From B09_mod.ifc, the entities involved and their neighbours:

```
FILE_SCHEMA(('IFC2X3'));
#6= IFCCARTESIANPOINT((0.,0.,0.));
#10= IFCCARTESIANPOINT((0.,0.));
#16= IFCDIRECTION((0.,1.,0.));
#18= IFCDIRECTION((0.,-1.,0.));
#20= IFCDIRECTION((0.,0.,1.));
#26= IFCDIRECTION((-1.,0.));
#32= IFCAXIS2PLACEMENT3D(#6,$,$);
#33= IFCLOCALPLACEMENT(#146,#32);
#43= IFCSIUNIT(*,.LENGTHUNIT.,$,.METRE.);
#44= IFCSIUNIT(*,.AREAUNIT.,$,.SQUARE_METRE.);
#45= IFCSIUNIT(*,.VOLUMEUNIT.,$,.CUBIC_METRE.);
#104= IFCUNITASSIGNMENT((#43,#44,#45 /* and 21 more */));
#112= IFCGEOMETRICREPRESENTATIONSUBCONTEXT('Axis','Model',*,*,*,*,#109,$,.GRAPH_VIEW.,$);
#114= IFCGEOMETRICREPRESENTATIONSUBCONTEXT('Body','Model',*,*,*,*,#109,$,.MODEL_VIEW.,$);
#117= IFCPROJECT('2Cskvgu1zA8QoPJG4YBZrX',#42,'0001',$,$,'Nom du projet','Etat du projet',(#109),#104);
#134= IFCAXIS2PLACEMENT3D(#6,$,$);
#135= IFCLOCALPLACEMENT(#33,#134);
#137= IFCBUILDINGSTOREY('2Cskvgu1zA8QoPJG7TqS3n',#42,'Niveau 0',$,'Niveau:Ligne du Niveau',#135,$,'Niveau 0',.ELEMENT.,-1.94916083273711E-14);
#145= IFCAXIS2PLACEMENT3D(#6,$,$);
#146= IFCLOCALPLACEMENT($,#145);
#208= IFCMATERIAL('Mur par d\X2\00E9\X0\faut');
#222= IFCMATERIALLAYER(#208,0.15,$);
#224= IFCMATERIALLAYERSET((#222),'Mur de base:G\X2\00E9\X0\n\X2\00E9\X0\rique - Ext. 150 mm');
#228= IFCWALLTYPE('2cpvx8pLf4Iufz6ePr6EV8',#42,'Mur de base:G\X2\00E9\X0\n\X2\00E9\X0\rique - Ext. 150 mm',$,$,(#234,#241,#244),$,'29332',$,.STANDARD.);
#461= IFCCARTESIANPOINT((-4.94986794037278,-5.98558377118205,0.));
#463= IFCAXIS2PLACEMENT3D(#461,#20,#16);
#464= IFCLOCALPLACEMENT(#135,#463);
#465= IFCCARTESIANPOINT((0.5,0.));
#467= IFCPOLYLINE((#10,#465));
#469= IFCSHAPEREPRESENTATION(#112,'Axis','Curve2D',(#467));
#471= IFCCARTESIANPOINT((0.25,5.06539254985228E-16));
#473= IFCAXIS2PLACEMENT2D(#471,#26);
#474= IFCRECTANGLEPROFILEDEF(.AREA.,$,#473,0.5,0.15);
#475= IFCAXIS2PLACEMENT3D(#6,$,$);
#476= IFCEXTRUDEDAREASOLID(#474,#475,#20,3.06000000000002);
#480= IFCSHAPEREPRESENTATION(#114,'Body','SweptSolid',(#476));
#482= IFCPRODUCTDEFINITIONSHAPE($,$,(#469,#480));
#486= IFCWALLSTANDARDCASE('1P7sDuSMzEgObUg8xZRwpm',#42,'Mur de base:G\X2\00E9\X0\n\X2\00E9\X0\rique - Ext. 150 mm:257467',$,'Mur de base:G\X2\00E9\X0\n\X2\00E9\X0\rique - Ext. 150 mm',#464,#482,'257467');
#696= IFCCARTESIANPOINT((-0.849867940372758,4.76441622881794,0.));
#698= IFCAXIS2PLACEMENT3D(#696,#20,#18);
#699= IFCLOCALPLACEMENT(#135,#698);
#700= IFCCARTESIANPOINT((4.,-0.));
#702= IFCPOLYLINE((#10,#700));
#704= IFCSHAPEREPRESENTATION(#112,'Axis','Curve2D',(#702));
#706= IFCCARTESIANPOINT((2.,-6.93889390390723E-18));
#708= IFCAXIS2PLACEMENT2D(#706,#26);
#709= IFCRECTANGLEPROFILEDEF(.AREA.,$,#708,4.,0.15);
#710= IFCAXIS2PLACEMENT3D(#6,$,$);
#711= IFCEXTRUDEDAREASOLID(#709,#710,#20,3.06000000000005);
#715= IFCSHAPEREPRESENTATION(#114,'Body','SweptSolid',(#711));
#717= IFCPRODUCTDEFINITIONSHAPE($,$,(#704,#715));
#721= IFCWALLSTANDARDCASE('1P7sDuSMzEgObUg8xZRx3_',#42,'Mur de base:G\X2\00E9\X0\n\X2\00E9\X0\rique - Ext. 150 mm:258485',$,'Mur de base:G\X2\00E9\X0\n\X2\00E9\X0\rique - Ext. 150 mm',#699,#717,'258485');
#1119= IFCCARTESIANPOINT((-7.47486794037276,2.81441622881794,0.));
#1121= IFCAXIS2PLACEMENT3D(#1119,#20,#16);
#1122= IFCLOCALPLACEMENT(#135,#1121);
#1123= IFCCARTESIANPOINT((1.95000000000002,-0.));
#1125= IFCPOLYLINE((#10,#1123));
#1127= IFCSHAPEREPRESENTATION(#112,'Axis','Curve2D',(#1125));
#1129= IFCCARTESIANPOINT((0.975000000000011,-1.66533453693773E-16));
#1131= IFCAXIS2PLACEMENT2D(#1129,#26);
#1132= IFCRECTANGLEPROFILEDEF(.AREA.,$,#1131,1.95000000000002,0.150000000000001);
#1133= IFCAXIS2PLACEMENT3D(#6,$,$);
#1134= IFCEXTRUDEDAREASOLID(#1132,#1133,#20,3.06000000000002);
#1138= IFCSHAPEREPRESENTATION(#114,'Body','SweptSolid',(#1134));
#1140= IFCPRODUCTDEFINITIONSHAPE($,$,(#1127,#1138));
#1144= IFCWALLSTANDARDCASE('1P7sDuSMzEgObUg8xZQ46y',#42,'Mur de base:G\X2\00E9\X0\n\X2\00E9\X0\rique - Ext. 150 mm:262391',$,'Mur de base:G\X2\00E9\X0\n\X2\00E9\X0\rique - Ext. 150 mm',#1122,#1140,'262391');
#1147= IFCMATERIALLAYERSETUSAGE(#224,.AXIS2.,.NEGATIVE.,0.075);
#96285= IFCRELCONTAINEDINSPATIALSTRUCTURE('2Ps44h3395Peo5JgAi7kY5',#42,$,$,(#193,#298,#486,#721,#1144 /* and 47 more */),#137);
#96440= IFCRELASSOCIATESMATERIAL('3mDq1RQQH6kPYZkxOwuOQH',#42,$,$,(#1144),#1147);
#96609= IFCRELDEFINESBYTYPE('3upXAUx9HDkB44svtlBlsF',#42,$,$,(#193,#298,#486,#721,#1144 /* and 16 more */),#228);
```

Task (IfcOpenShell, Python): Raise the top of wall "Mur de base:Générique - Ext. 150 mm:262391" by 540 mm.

```python
import ifcopenshell
import ifcopenshell.geom
import ifcopenshell.util.representation
import ifcopenshell.util.shape
import ifcopenshell.util.unit

model = ifcopenshell.open("B09_mod.ifc")
unit_scale = ifcopenshell.util.unit.calculate_unit_scale(model)
settings = ifcopenshell.geom.settings()


def volume(element):
    """Net volume in cubic metres, openings subtracted."""
    shape = ifcopenshell.geom.create_shape(settings, element)
    return ifcopenshell.util.shape.get_volume(shape.geometry)


wall = model.by_guid("1P7sDuSMzEgObUg8xZQ46y")
before = volume(wall)

body = ifcopenshell.util.representation.get_representation(wall, "Model", "Body")
solid = body.Items[0]
old_height = solid.Depth
solid.Depth += 0.54 / unit_scale
after = volume(wall)

print(f"height {old_height:g} -> {solid.Depth:g}, volume {before:.3f} -> {after:.3f} m3")

model.write("B09_mod_edited.ifc")
```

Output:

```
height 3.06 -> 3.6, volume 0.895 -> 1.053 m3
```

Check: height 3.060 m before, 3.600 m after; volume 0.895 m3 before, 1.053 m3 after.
